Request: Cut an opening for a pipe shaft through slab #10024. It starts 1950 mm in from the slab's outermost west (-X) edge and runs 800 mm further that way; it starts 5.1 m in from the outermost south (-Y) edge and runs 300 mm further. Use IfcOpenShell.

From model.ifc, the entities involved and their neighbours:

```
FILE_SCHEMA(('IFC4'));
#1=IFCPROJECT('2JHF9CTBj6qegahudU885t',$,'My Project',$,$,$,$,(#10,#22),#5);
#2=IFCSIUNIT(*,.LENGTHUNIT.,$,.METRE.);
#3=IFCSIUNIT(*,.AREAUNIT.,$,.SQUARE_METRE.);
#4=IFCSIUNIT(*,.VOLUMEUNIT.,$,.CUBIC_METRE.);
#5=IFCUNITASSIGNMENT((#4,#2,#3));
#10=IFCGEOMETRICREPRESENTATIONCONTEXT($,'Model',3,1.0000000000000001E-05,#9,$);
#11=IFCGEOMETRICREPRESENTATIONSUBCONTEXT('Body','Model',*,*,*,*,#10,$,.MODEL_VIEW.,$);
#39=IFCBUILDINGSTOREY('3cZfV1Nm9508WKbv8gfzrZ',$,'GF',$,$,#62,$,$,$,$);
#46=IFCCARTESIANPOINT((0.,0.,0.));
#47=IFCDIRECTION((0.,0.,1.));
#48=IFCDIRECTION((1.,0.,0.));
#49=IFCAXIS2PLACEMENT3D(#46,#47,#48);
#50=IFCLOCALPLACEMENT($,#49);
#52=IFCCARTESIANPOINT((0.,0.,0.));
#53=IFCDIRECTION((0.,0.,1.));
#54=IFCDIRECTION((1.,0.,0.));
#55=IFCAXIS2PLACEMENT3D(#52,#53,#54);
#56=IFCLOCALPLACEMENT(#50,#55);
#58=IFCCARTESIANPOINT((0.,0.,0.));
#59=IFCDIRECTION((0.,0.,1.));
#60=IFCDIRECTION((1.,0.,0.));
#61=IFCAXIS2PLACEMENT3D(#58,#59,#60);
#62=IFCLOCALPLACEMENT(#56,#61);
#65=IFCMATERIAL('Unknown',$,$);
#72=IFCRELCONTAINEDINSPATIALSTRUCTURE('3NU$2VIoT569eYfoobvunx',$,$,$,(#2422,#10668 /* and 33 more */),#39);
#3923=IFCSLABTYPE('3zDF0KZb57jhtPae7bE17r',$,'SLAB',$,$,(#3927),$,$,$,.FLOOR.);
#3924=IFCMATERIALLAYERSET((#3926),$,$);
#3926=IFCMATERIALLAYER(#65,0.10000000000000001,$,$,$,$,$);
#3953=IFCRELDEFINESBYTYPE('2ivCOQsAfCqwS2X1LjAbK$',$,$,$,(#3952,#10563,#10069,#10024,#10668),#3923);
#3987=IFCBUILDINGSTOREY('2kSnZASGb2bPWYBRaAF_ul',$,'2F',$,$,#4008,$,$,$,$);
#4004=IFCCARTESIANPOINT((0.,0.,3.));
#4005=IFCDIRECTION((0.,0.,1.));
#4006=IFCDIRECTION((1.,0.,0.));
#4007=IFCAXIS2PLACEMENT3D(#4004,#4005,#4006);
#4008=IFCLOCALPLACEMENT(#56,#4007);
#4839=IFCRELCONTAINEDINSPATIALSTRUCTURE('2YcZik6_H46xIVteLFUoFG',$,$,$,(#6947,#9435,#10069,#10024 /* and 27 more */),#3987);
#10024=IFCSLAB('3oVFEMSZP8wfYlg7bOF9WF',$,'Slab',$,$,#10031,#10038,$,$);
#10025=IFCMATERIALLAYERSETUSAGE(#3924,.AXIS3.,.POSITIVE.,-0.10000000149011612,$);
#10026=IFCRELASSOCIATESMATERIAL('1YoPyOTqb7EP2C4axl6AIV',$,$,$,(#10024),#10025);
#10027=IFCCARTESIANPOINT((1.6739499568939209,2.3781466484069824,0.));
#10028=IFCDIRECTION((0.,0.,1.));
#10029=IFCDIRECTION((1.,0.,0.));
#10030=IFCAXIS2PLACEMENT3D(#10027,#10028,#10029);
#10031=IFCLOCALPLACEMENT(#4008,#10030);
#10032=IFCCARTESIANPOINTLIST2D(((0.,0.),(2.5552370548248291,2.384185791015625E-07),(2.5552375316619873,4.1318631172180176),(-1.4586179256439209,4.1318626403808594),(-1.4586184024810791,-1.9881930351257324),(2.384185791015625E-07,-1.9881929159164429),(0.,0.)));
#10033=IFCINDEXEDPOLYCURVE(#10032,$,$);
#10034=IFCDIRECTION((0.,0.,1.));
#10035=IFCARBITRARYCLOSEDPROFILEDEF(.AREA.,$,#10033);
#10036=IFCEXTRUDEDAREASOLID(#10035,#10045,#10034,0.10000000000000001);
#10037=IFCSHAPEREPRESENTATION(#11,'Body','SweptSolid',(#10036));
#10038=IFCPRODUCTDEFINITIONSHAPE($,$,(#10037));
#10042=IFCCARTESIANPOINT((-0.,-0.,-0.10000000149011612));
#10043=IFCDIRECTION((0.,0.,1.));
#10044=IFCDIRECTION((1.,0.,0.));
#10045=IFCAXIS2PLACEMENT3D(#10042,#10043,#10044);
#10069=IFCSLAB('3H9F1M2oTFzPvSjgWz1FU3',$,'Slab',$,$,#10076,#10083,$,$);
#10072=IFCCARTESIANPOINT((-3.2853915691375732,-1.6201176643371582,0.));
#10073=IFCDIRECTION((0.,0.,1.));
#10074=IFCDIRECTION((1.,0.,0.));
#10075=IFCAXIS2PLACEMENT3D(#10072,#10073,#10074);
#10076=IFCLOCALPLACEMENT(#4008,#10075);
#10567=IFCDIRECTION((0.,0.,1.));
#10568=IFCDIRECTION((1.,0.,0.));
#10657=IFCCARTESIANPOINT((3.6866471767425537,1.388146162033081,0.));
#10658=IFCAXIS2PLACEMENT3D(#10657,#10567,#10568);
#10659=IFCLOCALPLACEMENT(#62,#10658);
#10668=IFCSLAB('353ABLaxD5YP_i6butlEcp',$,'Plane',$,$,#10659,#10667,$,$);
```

```python
import numpy as np
import ifcopenshell
import ifcopenshell.api.feature
import ifcopenshell.api.geometry
import ifcopenshell.api.root
import ifcopenshell.geom
import ifcopenshell.util.placement
import ifcopenshell.util.representation
import ifcopenshell.util.shape
import ifcopenshell.util.unit

model = ifcopenshell.open("model.ifc")
unit_scale = ifcopenshell.util.unit.calculate_unit_scale(model)
settings = ifcopenshell.geom.settings()


def volume(element):
    """Net volume in cubic metres, openings subtracted."""
    shape = ifcopenshell.geom.create_shape(settings, element)
    return ifcopenshell.util.shape.get_volume(shape.geometry)


slab = model.by_id(10024)
before = volume(slab)

# Extent in the slab's own axes, in metres. The edges named are its -X and -Y sides.
slab_shape = ifcopenshell.geom.create_shape(settings, slab)
vertices = ifcopenshell.util.shape.get_vertices(slab_shape.geometry)
x_min, y_min, bottom = vertices.min(axis=0)
top = vertices[:, 2].max()

opening = ifcopenshell.api.root.create_entity(model, ifc_class="IfcOpeningElement", name="Pipe shaft opening", predefined_type="OPENING")
context = ifcopenshell.util.representation.get_context(model, "Model", "Body", "MODEL_VIEW")
width, depth = 0.8, 0.3
outline = [(0.0, 0.0), (width, 0.0), (width, depth), (0.0, depth), (0.0, 0.0)]
# Overshoot both faces by 50 mm so the cut is clean.
shape = ifcopenshell.api.geometry.add_slab_representation(
    model, context=context, depth=top - bottom + 0.1, polyline=outline
)
ifcopenshell.api.geometry.assign_representation(model, product=opening, representation=shape)

matrix = ifcopenshell.util.placement.get_local_placement(slab.ObjectPlacement)
matrix[:, 3] = matrix @ np.append(np.array([x_min + 1.95, y_min + 5.1, bottom - 0.05]) / unit_scale, 1.0)
ifcopenshell.api.geometry.edit_object_placement(model, product=opening, matrix=matrix, is_si=False)
ifcopenshell.api.feature.add_feature(model, feature=opening, element=slab)

after = volume(slab)

print(f"slab volume {before:.3f} -> {after:.3f} m3")

model.write("model_updated.ifc")
```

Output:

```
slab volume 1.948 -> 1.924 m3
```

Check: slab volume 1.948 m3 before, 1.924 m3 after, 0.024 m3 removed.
